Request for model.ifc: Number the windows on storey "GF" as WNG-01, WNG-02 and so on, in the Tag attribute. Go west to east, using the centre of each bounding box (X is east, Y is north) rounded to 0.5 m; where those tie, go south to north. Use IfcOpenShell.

First a look at what the model holds.

```python
import ifcopenshell
import ifcopenshell.util.element
import ifcopenshell.util.placement

model = ifcopenshell.open("model.ifc")
print(model.schema)
storey = next(s for s in model.by_type("IfcBuildingStorey") if s.Name == "GF")
windows = [e for e in ifcopenshell.util.element.get_decomposition(storey) if e.is_a("IfcWindow")]
for e in sorted(windows, key=lambda e: e.id()):
    origin = ifcopenshell.util.placement.get_local_placement(e.ObjectPlacement)[:3, 3]
    print(e.id(), e.Tag, e.Name, origin.round(2) + 0.0, sep=" | ")
```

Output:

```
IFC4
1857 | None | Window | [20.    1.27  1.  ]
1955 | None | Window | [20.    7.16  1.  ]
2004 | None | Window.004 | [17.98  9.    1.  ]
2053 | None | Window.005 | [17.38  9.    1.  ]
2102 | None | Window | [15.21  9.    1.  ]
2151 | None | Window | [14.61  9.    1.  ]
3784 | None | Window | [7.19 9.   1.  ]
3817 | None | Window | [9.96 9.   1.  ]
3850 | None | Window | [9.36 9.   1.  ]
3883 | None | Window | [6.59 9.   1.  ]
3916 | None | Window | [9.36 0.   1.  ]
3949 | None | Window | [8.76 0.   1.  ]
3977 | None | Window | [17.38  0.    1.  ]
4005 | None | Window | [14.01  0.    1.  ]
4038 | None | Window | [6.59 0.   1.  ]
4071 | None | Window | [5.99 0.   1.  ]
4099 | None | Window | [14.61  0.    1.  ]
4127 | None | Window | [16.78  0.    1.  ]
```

```python
import ifcopenshell
import ifcopenshell.geom
import ifcopenshell.util.element
import ifcopenshell.util.shape

model = ifcopenshell.open("model.ifc")
settings = ifcopenshell.geom.settings()
settings.set("use-world-coords", True)


def centre(element):
    shape = ifcopenshell.geom.create_shape(settings, element)
    return ifcopenshell.util.shape.get_bbox_centroid(shape.geometry)


storey = next(s for s in model.by_type("IfcBuildingStorey") if s.Name == "GF")
windows = [e for e in ifcopenshell.util.element.get_decomposition(storey) if e.is_a("IfcWindow")]

# Insertion points can sit at a corner or the storey origin, so sort by the geometry (in metres).
centres = {e: centre(e) for e in windows}
windows.sort(key=lambda e: (round(centres[e][0] / 0.5), centres[e][1]))

for i, e in enumerate(windows, start=1):
    number = f"WNG-{i:02d}"
    e.Tag = number
    print(e.id(), number)

model.write("model_rev.ifc")
```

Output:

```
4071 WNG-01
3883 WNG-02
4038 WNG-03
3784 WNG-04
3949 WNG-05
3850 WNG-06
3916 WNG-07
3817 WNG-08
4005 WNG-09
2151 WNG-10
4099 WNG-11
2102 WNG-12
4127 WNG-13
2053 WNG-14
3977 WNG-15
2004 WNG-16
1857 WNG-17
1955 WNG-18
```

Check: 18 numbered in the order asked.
